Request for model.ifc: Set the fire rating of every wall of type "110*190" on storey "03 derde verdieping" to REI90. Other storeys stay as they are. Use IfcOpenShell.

First a look at what the model holds.

```python
import ifcopenshell
import ifcopenshell.util.element

model = ifcopenshell.open("model.ifc")
print(model.schema)
storey = next(s for s in model.by_type("IfcBuildingStorey") if s.Name == "03 derde verdieping")
walls = [e for e in ifcopenshell.util.element.get_decomposition(storey) if e.is_a("IfcWall")]
seen = {}
for e in walls:
    element_type = ifcopenshell.util.element.get_type(e)
    key = (element_type.Name if element_type != e and element_type else None, ifcopenshell.util.element.get_pset(e, "Pset_WallCommon", "FireRating"))
    seen[key] = seen.get(key, 0) + 1
for (name, value), count in sorted(seen.items(), key=str):
    print(count, "x", name, "|", value)
```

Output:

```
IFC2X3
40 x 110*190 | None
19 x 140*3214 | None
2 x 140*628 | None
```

```python
import ifcopenshell
import ifcopenshell.api.pset
import ifcopenshell.util.element

model = ifcopenshell.open("model.ifc")

storey = next(s for s in model.by_type("IfcBuildingStorey") if s.Name == "03 derde verdieping")
walls = [e for e in ifcopenshell.util.element.get_decomposition(storey) if e.is_a("IfcWall")]

count = 0
for e in walls:
    element_type = ifcopenshell.util.element.get_type(e)
    if element_type in (None, e) or element_type.Name != "110*190":
        continue
    found = ifcopenshell.util.element.get_pset(e, "Pset_WallCommon", should_inherit=False)
    if found:
        pset = model.by_id(found["id"])
        if len(ifcopenshell.util.element.get_elements_by_pset(pset)) > 1:
            pset = ifcopenshell.api.pset.unshare_pset(model, products=[e], pset=pset)[0]
    else:
        pset = ifcopenshell.api.pset.add_pset(model, product=e, name="Pset_WallCommon")
    ifcopenshell.api.pset.edit_pset(model, pset=pset, properties={"FireRating": "REI90"})
    count += 1

print(count, "walls updated")

model.write("model_v2.ifc")
```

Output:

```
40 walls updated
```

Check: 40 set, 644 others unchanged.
